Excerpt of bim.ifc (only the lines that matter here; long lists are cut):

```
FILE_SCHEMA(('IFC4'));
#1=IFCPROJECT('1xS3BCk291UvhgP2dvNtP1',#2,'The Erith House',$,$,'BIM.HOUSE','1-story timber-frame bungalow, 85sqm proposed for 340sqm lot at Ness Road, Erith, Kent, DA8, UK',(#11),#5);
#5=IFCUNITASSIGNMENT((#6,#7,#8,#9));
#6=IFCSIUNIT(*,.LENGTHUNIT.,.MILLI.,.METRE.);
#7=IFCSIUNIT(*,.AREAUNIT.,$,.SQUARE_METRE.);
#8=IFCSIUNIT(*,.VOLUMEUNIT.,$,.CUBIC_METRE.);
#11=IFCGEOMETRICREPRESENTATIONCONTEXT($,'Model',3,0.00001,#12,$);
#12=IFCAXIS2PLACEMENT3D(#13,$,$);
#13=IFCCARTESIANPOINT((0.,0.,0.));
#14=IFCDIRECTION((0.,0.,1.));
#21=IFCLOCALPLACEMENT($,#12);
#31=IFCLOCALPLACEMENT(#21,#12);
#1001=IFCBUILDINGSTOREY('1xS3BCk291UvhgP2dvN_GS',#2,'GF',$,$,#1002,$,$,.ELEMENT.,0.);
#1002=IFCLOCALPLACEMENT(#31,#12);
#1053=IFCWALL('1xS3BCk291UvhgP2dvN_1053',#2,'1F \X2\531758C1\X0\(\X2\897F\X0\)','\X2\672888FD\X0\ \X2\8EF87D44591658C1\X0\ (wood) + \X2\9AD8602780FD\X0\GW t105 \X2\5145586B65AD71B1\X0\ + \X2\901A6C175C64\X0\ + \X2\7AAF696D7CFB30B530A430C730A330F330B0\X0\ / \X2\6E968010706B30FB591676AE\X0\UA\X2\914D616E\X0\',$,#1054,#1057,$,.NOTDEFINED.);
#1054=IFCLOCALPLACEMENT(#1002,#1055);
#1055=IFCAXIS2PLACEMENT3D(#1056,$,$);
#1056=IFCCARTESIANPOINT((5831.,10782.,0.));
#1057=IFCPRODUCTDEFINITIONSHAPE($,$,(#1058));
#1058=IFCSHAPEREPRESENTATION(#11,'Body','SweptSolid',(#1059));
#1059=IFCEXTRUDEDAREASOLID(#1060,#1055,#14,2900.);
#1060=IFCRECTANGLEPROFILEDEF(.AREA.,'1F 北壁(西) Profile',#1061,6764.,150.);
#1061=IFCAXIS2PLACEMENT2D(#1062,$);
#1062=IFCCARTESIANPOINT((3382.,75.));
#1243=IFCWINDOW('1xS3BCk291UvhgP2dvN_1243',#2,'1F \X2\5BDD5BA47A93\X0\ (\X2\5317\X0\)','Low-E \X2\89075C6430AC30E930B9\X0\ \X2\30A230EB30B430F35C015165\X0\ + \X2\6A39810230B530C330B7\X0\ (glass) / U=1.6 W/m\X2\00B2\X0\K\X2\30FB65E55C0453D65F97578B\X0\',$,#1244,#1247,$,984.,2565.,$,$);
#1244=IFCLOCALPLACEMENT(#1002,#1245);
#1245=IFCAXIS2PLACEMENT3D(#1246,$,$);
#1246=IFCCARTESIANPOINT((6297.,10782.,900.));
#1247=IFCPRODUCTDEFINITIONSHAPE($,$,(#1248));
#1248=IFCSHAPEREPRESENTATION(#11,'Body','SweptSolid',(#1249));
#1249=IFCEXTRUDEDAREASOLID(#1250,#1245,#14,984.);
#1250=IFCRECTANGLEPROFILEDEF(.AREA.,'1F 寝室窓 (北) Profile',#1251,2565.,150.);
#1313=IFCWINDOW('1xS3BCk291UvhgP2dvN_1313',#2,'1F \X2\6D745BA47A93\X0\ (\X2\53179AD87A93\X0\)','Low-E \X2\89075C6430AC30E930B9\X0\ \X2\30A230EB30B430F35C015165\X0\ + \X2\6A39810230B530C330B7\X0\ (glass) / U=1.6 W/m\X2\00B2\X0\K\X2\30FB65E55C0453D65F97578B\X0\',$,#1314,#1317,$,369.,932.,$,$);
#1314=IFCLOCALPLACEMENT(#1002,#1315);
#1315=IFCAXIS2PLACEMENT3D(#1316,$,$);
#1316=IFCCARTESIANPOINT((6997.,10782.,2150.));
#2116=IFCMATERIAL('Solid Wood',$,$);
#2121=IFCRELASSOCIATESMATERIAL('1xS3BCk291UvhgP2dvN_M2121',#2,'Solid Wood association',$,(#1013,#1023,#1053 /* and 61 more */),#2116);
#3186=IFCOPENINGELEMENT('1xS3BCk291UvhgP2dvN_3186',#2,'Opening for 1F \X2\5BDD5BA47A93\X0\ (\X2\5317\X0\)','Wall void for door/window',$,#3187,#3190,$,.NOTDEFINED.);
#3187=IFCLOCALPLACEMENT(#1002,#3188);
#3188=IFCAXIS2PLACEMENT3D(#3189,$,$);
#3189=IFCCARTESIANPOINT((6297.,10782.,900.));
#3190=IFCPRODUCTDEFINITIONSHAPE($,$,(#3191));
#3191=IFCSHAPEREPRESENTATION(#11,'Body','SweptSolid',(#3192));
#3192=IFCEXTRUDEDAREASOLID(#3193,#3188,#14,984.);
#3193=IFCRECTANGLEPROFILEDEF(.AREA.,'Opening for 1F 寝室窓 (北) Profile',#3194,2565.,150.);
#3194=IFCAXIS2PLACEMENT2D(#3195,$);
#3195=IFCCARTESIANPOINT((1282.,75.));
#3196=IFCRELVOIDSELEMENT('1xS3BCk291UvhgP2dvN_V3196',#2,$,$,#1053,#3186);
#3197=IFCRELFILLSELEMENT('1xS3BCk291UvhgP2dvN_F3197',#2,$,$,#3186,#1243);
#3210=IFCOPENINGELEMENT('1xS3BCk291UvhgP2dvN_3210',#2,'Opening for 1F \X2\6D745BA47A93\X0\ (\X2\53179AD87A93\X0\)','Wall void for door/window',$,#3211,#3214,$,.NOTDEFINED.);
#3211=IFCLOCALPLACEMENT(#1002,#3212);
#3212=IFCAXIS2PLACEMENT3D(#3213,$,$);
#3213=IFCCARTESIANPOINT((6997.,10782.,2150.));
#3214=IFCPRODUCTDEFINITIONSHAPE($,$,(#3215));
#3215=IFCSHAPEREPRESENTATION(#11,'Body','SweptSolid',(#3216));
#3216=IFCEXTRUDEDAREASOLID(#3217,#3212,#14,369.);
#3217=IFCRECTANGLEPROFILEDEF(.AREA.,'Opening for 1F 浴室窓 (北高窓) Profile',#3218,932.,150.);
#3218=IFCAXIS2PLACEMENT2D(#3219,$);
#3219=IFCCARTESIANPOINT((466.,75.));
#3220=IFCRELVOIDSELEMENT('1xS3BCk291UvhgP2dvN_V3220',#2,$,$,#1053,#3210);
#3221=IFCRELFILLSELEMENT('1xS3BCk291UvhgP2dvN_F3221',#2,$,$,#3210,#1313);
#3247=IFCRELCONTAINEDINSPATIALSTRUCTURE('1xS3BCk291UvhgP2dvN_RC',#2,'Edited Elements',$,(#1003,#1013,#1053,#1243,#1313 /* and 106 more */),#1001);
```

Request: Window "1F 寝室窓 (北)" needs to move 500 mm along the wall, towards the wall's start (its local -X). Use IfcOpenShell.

```python
import ifcopenshell
import ifcopenshell.api.geometry
import ifcopenshell.util.placement
import ifcopenshell.util.unit

model = ifcopenshell.open("bim.ifc")
unit_scale = ifcopenshell.util.unit.calculate_unit_scale(model)

window = model.by_id(1243)
opening = window.FillsVoids[0].RelatingOpeningElement
wall = opening.VoidsElements[0].RelatingBuildingElement

wall_matrix = ifcopenshell.util.placement.get_local_placement(wall.ObjectPlacement)
shift = wall_matrix[:3, 0] * -0.5 / unit_scale
before = ifcopenshell.util.placement.get_local_placement(window.ObjectPlacement)[:3, 3].copy()

# The window is not placed relative to its opening, so move both.
for product in (opening, window):
    matrix = ifcopenshell.util.placement.get_local_placement(product.ObjectPlacement)
    matrix[:3, 3] += shift
    ifcopenshell.api.geometry.edit_object_placement(model, product=product, matrix=matrix, is_si=False)

after = ifcopenshell.util.placement.get_local_placement(window.ObjectPlacement)[:3, 3]
print("window moved by", (after - before).round(3) + 0.0)

model.write("bim_updated.ifc")
```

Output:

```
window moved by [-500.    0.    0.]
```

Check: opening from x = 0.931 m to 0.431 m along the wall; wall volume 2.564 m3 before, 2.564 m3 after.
